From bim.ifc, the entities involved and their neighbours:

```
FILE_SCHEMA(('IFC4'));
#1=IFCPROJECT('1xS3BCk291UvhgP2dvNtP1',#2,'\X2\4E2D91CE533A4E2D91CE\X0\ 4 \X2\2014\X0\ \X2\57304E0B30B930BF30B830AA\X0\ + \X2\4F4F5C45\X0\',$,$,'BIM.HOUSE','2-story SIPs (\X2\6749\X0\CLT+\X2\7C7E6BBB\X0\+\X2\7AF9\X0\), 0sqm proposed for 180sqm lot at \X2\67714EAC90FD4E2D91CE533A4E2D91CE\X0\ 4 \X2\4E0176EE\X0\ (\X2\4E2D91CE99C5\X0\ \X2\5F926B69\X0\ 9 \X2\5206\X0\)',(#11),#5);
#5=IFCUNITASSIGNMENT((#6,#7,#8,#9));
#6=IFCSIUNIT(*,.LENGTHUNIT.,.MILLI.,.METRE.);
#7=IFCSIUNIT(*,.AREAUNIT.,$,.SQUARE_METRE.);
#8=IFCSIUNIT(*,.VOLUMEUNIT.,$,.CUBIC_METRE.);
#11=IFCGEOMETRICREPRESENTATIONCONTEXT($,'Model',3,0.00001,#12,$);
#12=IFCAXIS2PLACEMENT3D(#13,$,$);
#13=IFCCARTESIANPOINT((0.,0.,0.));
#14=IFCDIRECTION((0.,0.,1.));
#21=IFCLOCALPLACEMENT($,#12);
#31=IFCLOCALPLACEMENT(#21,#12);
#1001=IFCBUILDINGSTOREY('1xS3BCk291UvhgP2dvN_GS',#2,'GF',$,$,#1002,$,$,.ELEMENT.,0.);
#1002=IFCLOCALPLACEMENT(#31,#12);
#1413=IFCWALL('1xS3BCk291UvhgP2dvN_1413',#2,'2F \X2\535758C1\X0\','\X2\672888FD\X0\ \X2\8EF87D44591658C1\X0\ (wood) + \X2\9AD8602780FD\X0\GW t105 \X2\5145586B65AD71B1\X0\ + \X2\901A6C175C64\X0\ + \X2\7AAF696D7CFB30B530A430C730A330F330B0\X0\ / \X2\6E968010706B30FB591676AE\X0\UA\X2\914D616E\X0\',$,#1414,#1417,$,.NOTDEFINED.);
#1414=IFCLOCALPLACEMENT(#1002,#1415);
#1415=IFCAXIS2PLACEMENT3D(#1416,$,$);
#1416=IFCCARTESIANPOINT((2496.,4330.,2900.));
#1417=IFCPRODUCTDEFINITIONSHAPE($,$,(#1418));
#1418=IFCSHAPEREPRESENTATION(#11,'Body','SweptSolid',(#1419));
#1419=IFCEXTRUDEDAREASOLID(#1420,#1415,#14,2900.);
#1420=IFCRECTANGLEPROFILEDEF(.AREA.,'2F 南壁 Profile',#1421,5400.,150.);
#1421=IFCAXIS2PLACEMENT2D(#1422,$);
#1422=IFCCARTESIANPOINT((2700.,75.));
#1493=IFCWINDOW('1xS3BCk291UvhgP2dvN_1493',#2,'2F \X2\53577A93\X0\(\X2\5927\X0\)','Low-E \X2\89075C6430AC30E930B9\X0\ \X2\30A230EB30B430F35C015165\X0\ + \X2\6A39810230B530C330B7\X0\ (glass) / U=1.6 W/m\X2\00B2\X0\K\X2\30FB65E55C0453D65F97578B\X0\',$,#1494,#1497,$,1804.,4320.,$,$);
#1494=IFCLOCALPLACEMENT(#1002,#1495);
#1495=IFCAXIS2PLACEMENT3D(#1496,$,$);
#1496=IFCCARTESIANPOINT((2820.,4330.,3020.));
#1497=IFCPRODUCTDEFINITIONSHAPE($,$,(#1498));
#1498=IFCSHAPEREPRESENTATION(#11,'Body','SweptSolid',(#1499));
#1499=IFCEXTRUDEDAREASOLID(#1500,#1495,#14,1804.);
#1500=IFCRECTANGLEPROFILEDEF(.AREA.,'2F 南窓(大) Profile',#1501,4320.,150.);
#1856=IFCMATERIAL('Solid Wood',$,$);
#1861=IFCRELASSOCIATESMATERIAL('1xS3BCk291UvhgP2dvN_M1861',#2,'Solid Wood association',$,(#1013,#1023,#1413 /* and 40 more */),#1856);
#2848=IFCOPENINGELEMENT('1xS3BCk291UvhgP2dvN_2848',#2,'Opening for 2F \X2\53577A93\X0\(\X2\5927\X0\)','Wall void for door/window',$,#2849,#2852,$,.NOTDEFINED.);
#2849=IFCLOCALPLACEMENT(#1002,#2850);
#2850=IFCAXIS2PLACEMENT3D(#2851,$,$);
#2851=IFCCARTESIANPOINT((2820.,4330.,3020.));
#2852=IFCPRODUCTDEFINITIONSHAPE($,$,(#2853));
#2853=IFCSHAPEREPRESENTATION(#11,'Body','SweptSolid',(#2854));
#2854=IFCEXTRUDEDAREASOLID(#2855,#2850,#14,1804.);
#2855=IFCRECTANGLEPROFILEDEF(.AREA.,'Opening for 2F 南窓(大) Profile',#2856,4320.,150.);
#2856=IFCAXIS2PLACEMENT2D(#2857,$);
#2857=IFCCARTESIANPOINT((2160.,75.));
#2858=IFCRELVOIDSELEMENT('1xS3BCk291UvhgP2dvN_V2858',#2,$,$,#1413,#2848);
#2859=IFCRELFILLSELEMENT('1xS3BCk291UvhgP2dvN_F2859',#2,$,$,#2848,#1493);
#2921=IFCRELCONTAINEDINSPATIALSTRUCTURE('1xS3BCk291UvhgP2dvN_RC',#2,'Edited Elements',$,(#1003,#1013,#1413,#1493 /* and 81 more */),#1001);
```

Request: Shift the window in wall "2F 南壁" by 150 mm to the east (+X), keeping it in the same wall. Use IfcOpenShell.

```python
import ifcopenshell
import ifcopenshell.api.geometry
import ifcopenshell.util.placement
import ifcopenshell.util.unit

model = ifcopenshell.open("bim.ifc")
unit_scale = ifcopenshell.util.unit.calculate_unit_scale(model)

window = model.by_guid("1xS3BCk291UvhgP2dvN_1493")
opening = window.FillsVoids[0].RelatingOpeningElement
wall = opening.VoidsElements[0].RelatingBuildingElement

wall_matrix = ifcopenshell.util.placement.get_local_placement(wall.ObjectPlacement)
shift = wall_matrix[:3, 0] * 0.15 / unit_scale
before = ifcopenshell.util.placement.get_local_placement(window.ObjectPlacement)[:3, 3].copy()

# The window is not placed relative to its opening, so move both.
for product in (opening, window):
    matrix = ifcopenshell.util.placement.get_local_placement(product.ObjectPlacement)
    matrix[:3, 3] += shift
    ifcopenshell.api.geometry.edit_object_placement(model, product=product, matrix=matrix, is_si=False)

after = ifcopenshell.util.placement.get_local_placement(window.ObjectPlacement)[:3, 3]
print("window moved by", (after - before).round(3) + 0.0)

model.write("bim_v2.ifc")
```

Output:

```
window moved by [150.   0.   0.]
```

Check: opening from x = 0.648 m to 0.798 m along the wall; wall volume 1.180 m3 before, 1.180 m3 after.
